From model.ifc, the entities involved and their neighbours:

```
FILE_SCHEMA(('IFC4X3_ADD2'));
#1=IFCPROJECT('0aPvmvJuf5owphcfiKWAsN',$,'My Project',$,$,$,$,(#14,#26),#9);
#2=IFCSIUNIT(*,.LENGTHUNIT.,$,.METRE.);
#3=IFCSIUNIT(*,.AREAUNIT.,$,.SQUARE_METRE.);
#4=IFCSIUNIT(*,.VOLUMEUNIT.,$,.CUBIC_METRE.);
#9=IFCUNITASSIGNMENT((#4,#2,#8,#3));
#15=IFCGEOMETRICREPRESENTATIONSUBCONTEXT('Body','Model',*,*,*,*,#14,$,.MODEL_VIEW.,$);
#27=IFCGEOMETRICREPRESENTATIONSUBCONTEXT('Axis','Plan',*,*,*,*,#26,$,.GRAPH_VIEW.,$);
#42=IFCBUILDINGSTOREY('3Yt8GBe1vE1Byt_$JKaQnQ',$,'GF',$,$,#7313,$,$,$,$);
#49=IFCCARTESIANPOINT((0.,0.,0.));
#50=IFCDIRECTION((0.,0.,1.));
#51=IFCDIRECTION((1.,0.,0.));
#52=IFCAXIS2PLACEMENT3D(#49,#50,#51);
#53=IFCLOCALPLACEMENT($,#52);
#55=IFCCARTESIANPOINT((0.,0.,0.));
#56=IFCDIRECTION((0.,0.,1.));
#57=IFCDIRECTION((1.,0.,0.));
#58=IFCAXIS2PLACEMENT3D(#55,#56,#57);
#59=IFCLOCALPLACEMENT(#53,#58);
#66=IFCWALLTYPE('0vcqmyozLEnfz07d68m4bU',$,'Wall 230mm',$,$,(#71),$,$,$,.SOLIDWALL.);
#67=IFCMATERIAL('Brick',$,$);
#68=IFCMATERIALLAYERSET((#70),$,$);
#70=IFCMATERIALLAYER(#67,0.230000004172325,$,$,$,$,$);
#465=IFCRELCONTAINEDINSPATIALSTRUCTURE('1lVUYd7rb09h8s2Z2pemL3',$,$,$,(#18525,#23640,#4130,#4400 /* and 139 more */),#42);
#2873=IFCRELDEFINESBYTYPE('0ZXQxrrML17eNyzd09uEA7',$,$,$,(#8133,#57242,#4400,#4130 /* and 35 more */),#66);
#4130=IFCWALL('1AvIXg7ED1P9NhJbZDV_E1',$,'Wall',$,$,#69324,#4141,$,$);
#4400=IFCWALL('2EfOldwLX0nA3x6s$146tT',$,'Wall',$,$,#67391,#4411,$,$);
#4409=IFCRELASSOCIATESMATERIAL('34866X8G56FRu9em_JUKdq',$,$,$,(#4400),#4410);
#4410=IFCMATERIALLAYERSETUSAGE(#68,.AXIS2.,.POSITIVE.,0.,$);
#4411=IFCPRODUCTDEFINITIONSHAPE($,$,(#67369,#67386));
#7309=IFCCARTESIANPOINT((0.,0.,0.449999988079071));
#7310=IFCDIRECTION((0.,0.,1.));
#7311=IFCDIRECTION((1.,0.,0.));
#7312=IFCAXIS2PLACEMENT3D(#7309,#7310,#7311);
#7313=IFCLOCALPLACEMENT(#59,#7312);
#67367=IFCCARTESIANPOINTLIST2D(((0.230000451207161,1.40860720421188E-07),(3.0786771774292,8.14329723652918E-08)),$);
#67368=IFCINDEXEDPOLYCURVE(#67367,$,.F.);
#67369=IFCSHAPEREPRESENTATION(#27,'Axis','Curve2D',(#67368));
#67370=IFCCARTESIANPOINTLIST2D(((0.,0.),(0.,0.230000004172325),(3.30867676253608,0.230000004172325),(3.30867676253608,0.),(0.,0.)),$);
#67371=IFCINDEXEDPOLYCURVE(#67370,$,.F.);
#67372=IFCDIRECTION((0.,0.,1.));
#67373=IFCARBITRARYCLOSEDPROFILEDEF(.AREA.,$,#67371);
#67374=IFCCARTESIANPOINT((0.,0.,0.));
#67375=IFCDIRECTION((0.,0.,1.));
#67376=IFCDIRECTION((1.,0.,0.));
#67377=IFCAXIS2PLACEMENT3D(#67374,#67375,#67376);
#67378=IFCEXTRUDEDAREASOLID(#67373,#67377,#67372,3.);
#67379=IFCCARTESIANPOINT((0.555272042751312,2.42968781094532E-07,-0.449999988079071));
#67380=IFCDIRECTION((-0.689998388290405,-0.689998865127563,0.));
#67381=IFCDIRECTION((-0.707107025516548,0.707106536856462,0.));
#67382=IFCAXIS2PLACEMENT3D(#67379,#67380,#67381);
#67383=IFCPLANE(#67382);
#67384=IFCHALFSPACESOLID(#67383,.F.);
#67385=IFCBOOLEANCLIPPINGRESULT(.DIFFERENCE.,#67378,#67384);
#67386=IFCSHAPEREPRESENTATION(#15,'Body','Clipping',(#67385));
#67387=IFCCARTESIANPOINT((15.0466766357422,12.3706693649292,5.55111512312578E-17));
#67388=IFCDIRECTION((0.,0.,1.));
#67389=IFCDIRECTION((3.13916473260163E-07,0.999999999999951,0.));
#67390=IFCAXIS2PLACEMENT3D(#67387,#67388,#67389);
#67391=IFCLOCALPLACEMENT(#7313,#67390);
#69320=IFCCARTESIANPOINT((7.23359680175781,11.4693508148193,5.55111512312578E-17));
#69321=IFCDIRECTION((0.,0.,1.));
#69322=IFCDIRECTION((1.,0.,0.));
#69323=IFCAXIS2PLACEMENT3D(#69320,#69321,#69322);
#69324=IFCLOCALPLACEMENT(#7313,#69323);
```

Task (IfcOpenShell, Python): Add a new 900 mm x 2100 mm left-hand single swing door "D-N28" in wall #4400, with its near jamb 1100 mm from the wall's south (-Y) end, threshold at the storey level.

```python
import numpy as np
import ifcopenshell
import ifcopenshell.api.feature
import ifcopenshell.api.geometry
import ifcopenshell.api.root
import ifcopenshell.api.spatial
import ifcopenshell.geom
import ifcopenshell.util.element
import ifcopenshell.util.placement
import ifcopenshell.util.representation
import ifcopenshell.util.shape
import ifcopenshell.util.unit

model = ifcopenshell.open("model.ifc")
unit_scale = ifcopenshell.util.unit.calculate_unit_scale(model)
settings = ifcopenshell.geom.settings()


def volume(element):
    """Net volume in cubic metres, openings subtracted."""
    shape = ifcopenshell.geom.create_shape(settings, element)
    return ifcopenshell.util.shape.get_volume(shape.geometry)


wall = model.by_guid("2EfOldwLX0nA3x6s$146tT")
storey = ifcopenshell.util.element.get_container(wall, ifc_class="IfcBuildingStorey")
context = ifcopenshell.util.representation.get_context(model, "Model", "Body", "MODEL_VIEW")
before = volume(wall)

width, height, from_end, sill = 0.9, 2.1, 1.1, 0.0  # metres

# The wall runs along its own X axis, and the end named is its -X end.
wall_shape = ifcopenshell.geom.create_shape(settings, wall)
x, y, z = ifcopenshell.util.shape.get_vertices(wall_shape.geometry).T
start = x.min() + from_end
face, thickness = float(y.min()), float(y.max() - y.min())
wall_matrix = ifcopenshell.util.placement.get_local_placement(wall.ObjectPlacement)
level = ifcopenshell.util.placement.get_local_placement(storey.ObjectPlacement)[2, 3]


def in_wall(x, y):
    """Placement at x, y metres in the wall's axes, at sill height."""
    matrix = wall_matrix.copy()
    matrix[:, 3] = wall_matrix @ np.array([x / unit_scale, y / unit_scale, 0.0, 1.0])
    matrix[2, 3] = level + sill / unit_scale
    return matrix


# Opening: a box that overshoots both wall faces by 50 mm.
opening = ifcopenshell.api.root.create_entity(model, ifc_class="IfcOpeningElement", predefined_type="OPENING")
box = ifcopenshell.api.geometry.add_wall_representation(
    model, context=context, length=width, height=height, thickness=thickness + 0.1
)
ifcopenshell.api.geometry.assign_representation(model, product=opening, representation=box)
ifcopenshell.api.geometry.edit_object_placement(model, product=opening, matrix=in_wall(start, face - 0.05), is_si=False)
ifcopenshell.api.feature.add_feature(model, feature=opening, element=wall)

door = ifcopenshell.api.root.create_entity(model, ifc_class="IfcDoor", name="D-N28", predefined_type="DOOR")
door.OverallWidth, door.OverallHeight = width / unit_scale, height / unit_scale
door.OperationType = "SINGLE_SWING_LEFT"
body = ifcopenshell.api.geometry.add_door_representation(
    model,
    context=context,
    overall_width=door.OverallWidth,
    overall_height=door.OverallHeight,
    operation_type="SINGLE_SWING_LEFT",
    lining_properties={"LiningDepth": thickness / unit_scale, "ThresholdDepth": thickness / unit_scale},
)
ifcopenshell.api.geometry.assign_representation(model, product=door, representation=body)
ifcopenshell.api.spatial.assign_container(model, products=[door], relating_structure=storey)
ifcopenshell.api.feature.add_filling(model, opening=opening, element=door)

# The lining spans the wall, so the door starts at the wall face.
ifcopenshell.api.geometry.edit_object_placement(model, product=door, matrix=in_wall(start, face), is_si=False)

after = volume(wall)

print(f"wall volume {before:.3f} -> {after:.3f} m3")

model.write("model_rev.ifc")
```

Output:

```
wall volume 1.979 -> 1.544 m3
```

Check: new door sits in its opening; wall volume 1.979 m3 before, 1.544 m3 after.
